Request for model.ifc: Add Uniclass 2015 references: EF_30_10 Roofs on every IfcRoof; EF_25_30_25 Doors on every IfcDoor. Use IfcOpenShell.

First a look at what the model holds.

```python
import ifcopenshell

model = ifcopenshell.open("model.ifc")
print(model.schema)
print("classifications:", [c.Name for c in model.by_type("IfcClassification")])
for ifc_class in ("IfcDoor", "IfcRoof", "IfcStair", "IfcWall", "IfcWindow"):
    print(ifc_class, len(model.by_type(ifc_class)))
```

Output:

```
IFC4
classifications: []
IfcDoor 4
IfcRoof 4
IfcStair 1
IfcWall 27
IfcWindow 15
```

```python
import ifcopenshell
import ifcopenshell.api.classification

model = ifcopenshell.open("model.ifc")

system = ifcopenshell.api.classification.add_classification(model, classification="Uniclass 2015")

codes = {
    "IfcRoof": ("EF_30_10", "Roofs"),
    "IfcDoor": ("EF_25_30_25", "Doors"),
}
for ifc_class, (code, name) in codes.items():
    products = model.by_type(ifc_class)
    ifcopenshell.api.classification.add_reference(
        model, products=products, classification=system, identification=code, name=name
    )
    print(code, len(products))

model.write("model_v2.ifc")
```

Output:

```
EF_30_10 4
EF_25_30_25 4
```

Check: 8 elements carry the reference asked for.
